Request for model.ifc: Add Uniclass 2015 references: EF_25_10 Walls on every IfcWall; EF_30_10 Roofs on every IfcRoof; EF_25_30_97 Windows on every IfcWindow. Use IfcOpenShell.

First a look at what the model holds.

```python
import ifcopenshell

model = ifcopenshell.open("model.ifc")
print(model.schema)
print("classifications:", [c.Name for c in model.by_type("IfcClassification")])
for ifc_class in ("IfcDoor", "IfcRoof", "IfcStair", "IfcWall", "IfcWindow"):
    print(ifc_class, len(model.by_type(ifc_class)))
```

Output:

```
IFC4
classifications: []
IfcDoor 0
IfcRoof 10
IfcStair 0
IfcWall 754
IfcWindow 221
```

```python
import ifcopenshell
import ifcopenshell.api.classification

model = ifcopenshell.open("model.ifc")

system = ifcopenshell.api.classification.add_classification(model, classification="Uniclass 2015")

codes = {
    "IfcWall": ("EF_25_10", "Walls"),
    "IfcRoof": ("EF_30_10", "Roofs"),
    "IfcWindow": ("EF_25_30_97", "Windows"),
}
for ifc_class, (code, name) in codes.items():
    products = model.by_type(ifc_class)
    ifcopenshell.api.classification.add_reference(
        model, products=products, classification=system, identification=code, name=name
    )
    print(code, len(products))

model.write("model_updated.ifc")
```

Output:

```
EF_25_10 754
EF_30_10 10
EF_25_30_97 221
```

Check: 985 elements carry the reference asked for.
